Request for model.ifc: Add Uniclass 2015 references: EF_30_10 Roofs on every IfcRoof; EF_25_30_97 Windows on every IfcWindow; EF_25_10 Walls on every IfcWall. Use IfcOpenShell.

First a look at what the model holds.

```python
import ifcopenshell

model = ifcopenshell.open("model.ifc")
print(model.schema)
print("classifications:", [c.Name for c in model.by_type("IfcClassification")])
for ifc_class in ("IfcDoor", "IfcRoof", "IfcStair", "IfcWall", "IfcWindow"):
    print(ifc_class, len(model.by_type(ifc_class)))
```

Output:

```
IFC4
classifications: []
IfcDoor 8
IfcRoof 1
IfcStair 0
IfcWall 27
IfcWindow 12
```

```python
import ifcopenshell
import ifcopenshell.api.classification

model = ifcopenshell.open("model.ifc")

system = ifcopenshell.api.classification.add_classification(model, classification="Uniclass 2015")

codes = {
    "IfcRoof": ("EF_30_10", "Roofs"),
    "IfcWindow": ("EF_25_30_97", "Windows"),
    "IfcWall": ("EF_25_10", "Walls"),
}
for ifc_class, (code, name) in codes.items():
    products = model.by_type(ifc_class)
    ifcopenshell.api.classification.add_reference(
        model, products=products, classification=system, identification=code, name=name
    )
    print(code, len(products))

model.write("model_edited.ifc")
```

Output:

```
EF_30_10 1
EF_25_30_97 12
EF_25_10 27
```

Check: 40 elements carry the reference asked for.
